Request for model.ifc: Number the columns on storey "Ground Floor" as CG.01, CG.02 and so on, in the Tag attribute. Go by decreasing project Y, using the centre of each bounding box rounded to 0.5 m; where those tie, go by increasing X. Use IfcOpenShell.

First a look at what the model holds.

```python
import ifcopenshell
import ifcopenshell.util.element
import ifcopenshell.util.placement

model = ifcopenshell.open("model.ifc")
print(model.schema)
storey = next(s for s in model.by_type("IfcBuildingStorey") if s.Name == "Ground Floor")
columns = [e for e in ifcopenshell.util.element.get_decomposition(storey) if e.is_a("IfcColumn")]
for e in sorted(columns, key=lambda e: e.id()):
    origin = ifcopenshell.util.placement.get_local_placement(e.ObjectPlacement)[:3, 3]
    print(e.id(), e.Tag, e.Name, origin.round(2) + 0.0, sep=" | ")
```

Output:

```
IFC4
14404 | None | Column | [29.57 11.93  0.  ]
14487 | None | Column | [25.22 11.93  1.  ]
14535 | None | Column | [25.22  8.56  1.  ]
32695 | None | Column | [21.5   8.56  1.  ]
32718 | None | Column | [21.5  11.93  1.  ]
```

```python
import ifcopenshell
import ifcopenshell.geom
import ifcopenshell.util.element
import ifcopenshell.util.shape

model = ifcopenshell.open("model.ifc")
settings = ifcopenshell.geom.settings()
settings.set("use-world-coords", True)


def centre(element):
    shape = ifcopenshell.geom.create_shape(settings, element)
    return ifcopenshell.util.shape.get_bbox_centroid(shape.geometry)


storey = next(s for s in model.by_type("IfcBuildingStorey") if s.Name == "Ground Floor")
columns = [e for e in ifcopenshell.util.element.get_decomposition(storey) if e.is_a("IfcColumn")]

# Insertion points can sit at a corner or the storey origin, so sort by the geometry (in metres).
centres = {e: centre(e) for e in columns}
columns.sort(key=lambda e: (-round(centres[e][1] / 0.5), centres[e][0]))

for i, e in enumerate(columns, start=1):
    number = f"CG.{i:02d}"
    e.Tag = number
    print(e.id(), number)

model.write("model_rev.ifc")
```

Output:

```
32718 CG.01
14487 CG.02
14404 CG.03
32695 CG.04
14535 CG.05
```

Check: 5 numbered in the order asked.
